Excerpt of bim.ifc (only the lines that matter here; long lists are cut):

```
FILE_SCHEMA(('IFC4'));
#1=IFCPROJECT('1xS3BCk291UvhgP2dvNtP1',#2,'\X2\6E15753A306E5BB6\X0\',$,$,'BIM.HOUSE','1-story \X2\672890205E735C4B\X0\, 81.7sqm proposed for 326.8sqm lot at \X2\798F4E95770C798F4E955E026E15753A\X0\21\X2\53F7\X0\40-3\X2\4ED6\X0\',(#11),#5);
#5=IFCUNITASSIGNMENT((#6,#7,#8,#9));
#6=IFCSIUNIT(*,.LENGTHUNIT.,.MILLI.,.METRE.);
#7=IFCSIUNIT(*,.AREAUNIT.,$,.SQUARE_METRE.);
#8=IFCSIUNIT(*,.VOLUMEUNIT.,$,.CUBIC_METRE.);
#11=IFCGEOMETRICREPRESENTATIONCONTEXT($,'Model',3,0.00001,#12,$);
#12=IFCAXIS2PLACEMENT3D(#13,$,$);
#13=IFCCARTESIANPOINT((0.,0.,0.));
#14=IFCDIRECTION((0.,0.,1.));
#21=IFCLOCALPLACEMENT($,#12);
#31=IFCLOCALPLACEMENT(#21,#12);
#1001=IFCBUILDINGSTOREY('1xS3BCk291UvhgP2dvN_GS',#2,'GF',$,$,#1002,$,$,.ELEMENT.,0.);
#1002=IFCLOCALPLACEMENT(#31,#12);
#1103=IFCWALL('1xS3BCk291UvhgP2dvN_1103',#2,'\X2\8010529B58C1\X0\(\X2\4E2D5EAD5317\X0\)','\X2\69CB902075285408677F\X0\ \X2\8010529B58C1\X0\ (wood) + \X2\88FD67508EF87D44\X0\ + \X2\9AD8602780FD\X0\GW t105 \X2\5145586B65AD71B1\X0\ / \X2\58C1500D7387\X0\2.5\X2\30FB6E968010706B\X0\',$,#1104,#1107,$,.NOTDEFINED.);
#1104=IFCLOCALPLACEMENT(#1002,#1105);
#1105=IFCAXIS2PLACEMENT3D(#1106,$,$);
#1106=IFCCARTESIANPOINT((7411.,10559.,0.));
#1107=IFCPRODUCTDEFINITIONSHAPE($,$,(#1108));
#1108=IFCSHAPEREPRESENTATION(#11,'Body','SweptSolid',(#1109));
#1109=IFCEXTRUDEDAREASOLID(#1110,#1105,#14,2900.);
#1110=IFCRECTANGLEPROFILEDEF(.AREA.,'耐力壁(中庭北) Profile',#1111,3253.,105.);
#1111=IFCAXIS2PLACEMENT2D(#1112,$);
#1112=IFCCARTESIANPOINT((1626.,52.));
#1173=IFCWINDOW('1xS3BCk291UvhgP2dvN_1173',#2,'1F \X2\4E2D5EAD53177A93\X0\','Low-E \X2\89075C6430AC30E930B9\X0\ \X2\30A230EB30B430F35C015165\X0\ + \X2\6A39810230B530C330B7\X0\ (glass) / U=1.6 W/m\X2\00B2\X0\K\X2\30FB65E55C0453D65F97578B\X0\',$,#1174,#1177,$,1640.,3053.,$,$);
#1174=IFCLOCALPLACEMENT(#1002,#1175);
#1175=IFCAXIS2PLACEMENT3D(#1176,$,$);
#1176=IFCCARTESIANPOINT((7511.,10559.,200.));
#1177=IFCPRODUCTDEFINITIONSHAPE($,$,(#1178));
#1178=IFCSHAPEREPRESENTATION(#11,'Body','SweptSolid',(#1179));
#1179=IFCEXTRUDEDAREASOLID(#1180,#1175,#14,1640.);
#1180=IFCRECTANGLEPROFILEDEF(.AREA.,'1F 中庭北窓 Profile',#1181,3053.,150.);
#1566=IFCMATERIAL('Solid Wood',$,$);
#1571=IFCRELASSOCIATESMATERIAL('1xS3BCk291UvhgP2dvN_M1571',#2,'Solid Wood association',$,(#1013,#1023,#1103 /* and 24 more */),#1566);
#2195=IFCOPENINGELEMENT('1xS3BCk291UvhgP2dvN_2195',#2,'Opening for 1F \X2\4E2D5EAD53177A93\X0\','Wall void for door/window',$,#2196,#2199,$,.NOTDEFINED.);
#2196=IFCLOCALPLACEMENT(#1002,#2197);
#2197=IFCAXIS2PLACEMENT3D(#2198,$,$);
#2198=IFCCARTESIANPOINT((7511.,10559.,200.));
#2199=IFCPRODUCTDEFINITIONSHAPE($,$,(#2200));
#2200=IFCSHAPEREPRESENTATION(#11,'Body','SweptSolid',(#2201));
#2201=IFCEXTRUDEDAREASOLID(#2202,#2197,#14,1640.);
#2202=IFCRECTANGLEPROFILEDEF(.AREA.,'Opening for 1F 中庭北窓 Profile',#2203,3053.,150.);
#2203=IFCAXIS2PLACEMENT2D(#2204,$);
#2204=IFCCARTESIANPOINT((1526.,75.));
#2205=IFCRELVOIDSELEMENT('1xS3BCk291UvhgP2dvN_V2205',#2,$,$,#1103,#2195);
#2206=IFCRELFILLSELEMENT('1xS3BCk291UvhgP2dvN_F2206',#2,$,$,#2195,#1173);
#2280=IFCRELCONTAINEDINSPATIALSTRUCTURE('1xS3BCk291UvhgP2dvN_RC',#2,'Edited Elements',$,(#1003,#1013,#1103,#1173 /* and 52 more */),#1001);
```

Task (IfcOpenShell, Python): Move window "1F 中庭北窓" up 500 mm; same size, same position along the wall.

```python
import numpy as np
import ifcopenshell
import ifcopenshell.api.geometry
import ifcopenshell.util.placement
import ifcopenshell.util.unit

model = ifcopenshell.open("bim.ifc")
unit_scale = ifcopenshell.util.unit.calculate_unit_scale(model)

window = model.by_guid("1xS3BCk291UvhgP2dvN_1173")
opening = window.FillsVoids[0].RelatingOpeningElement
dz = 500.0

shift = np.array([0.0, 0.0, dz])
# The window is not placed relative to its opening, so move both.
for product in (opening, window):
    matrix = ifcopenshell.util.placement.get_local_placement(product.ObjectPlacement)
    matrix[:3, 3] += shift
    ifcopenshell.api.geometry.edit_object_placement(model, product=product, matrix=matrix, is_si=False)

print(f"moved by {dz * unit_scale:+.3f} m")

model.write("bim-out.ifc")
```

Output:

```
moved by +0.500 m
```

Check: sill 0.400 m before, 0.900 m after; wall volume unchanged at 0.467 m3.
